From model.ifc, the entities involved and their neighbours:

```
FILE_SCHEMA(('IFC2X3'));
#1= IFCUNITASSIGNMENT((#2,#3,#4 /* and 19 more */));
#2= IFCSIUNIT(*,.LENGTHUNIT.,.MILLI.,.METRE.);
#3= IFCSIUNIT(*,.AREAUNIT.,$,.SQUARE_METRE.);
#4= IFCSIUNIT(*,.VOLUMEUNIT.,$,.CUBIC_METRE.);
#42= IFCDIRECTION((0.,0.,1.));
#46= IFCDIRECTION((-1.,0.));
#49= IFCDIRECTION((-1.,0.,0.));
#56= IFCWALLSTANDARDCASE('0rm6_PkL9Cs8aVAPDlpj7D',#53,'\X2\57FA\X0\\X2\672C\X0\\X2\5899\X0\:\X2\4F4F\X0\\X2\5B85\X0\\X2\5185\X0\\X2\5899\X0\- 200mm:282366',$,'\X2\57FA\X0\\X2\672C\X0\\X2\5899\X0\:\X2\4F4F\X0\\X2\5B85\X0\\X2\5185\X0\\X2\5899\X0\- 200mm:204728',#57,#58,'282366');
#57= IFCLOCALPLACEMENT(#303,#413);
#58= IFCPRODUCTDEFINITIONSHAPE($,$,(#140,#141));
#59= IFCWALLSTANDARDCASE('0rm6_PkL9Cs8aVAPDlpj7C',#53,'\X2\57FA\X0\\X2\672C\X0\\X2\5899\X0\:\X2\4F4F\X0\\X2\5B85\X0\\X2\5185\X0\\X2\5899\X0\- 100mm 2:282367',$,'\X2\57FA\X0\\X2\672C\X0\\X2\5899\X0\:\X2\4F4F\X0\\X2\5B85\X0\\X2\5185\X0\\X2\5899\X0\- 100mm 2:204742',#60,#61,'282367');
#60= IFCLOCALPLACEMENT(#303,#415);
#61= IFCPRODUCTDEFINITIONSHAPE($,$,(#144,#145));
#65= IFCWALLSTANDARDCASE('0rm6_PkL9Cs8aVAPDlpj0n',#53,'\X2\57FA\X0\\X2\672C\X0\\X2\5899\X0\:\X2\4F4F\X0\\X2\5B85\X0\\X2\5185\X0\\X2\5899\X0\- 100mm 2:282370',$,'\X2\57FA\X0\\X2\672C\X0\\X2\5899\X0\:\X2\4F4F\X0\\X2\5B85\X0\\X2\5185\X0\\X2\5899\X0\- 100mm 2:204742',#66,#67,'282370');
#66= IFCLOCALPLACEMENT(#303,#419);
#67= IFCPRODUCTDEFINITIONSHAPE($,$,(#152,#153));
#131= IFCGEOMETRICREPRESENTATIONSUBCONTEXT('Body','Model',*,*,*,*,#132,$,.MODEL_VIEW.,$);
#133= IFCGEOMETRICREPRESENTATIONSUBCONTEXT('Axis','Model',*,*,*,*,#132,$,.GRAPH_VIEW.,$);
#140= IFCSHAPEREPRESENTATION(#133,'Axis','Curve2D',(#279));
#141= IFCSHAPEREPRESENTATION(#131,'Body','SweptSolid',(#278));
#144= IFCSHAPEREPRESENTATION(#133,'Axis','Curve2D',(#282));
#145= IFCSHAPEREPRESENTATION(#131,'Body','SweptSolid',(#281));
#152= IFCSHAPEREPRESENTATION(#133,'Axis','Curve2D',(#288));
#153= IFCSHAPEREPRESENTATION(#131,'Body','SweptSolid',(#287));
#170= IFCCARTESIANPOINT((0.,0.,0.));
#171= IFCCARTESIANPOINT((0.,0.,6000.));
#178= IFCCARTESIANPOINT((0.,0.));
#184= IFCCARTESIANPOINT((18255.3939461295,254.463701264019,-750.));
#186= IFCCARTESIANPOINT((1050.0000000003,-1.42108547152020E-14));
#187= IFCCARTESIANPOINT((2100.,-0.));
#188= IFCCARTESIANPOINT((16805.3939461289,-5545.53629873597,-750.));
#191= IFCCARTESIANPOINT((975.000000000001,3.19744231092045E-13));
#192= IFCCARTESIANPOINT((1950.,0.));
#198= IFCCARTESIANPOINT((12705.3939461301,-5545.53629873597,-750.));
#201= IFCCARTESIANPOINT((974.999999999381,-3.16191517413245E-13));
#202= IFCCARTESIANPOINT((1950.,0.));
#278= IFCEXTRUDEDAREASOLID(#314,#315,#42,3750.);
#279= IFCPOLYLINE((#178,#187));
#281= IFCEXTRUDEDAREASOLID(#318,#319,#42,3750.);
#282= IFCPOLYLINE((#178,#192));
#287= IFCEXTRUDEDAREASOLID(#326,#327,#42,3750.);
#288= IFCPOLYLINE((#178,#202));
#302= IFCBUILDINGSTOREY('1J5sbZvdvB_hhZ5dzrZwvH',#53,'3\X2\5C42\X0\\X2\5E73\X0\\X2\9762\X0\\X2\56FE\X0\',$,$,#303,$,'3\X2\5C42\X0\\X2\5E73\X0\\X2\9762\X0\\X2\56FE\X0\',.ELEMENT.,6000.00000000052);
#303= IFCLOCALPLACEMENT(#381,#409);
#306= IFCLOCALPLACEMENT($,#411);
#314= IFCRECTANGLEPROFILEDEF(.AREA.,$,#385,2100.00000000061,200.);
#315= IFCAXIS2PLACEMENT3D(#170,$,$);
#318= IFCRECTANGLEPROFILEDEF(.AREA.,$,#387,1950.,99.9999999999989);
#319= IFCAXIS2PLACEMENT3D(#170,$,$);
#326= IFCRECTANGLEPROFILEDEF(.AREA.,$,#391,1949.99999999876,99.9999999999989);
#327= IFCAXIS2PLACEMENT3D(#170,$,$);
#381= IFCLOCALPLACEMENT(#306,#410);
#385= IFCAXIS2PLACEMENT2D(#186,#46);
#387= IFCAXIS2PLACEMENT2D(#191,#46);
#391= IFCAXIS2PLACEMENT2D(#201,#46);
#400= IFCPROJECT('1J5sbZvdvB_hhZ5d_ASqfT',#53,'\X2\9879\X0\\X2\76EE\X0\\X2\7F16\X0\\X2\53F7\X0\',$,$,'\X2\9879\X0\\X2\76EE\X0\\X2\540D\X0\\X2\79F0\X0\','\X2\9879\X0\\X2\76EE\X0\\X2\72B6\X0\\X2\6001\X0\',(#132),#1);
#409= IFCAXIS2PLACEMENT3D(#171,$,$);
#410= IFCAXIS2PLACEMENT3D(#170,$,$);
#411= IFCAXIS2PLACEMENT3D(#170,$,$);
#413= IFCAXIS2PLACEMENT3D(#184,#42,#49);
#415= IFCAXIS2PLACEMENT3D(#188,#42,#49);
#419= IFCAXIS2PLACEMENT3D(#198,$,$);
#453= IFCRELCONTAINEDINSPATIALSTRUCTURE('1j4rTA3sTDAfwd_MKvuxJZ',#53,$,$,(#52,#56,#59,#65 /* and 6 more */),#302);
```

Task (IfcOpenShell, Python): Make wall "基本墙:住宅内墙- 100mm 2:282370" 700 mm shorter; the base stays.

```python
import ifcopenshell
import ifcopenshell.geom
import ifcopenshell.util.representation
import ifcopenshell.util.shape
import ifcopenshell.util.unit

model = ifcopenshell.open("model.ifc")
unit_scale = ifcopenshell.util.unit.calculate_unit_scale(model)
settings = ifcopenshell.geom.settings()


def volume(element):
    """Net volume in cubic metres, openings subtracted."""
    shape = ifcopenshell.geom.create_shape(settings, element)
    return ifcopenshell.util.shape.get_volume(shape.geometry)


wall = model.by_guid("0rm6_PkL9Cs8aVAPDlpj0n")
before = volume(wall)

body = ifcopenshell.util.representation.get_representation(wall, "Model", "Body")
solid = body.Items[0]
old_height = solid.Depth
solid.Depth -= 0.7 / unit_scale
after = volume(wall)

print(f"height {old_height:g} -> {solid.Depth:g}, volume {before:.3f} -> {after:.3f} m3")

model.write("model_edited.ifc")
```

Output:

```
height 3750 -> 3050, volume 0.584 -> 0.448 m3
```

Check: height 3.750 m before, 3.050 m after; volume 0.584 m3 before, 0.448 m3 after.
